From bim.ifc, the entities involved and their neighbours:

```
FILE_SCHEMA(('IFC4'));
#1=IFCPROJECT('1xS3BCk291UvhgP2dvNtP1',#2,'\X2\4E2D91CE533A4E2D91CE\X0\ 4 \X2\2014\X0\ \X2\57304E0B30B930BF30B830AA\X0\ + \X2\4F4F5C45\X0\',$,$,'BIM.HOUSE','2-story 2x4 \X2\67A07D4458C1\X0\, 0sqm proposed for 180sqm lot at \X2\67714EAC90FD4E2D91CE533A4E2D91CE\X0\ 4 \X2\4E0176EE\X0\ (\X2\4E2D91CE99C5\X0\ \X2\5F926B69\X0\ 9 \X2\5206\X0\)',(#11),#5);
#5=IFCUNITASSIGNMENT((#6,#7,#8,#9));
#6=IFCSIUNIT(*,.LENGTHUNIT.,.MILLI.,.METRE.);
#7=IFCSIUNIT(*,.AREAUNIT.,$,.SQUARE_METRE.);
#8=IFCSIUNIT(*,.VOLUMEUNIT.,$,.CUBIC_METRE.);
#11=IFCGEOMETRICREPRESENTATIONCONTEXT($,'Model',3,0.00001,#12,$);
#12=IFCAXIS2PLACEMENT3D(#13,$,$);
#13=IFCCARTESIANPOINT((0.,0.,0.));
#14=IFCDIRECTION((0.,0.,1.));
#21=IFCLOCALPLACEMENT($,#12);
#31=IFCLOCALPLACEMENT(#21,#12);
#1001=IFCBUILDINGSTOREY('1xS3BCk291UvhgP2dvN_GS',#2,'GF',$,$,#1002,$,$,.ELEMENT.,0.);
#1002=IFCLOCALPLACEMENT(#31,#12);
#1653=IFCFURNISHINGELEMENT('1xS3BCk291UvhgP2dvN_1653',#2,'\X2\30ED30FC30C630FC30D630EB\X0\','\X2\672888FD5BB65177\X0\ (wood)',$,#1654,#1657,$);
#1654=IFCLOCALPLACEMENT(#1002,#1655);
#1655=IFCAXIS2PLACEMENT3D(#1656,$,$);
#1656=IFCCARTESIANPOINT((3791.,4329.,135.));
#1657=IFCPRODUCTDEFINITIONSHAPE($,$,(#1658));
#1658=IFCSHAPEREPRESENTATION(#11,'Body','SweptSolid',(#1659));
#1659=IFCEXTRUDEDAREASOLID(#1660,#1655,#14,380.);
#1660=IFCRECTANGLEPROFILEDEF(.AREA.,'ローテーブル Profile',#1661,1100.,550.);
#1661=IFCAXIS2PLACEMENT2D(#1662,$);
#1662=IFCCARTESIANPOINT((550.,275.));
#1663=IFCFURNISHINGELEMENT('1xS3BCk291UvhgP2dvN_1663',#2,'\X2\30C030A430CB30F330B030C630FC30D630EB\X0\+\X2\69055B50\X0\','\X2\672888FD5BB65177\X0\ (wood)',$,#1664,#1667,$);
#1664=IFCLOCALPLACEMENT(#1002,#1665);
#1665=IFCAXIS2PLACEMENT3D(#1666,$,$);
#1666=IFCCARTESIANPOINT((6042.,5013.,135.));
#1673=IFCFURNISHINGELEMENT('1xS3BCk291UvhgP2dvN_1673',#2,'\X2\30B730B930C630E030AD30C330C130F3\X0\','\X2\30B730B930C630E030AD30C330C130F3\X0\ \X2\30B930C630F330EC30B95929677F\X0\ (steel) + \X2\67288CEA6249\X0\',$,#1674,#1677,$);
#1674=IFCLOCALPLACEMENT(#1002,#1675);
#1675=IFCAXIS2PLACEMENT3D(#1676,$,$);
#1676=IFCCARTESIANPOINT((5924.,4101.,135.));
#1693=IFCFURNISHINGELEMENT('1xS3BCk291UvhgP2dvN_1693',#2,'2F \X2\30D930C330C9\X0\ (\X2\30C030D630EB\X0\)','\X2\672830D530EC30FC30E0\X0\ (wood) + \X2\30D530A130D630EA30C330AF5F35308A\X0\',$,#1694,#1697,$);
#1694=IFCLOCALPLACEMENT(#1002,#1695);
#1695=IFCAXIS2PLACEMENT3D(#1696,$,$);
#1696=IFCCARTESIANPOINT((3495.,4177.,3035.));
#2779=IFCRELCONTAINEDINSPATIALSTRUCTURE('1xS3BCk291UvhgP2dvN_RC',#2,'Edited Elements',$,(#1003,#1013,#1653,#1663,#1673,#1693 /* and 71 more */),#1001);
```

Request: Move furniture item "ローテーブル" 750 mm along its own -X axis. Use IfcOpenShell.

```python
import ifcopenshell
import ifcopenshell.api.geometry
import ifcopenshell.util.placement
import ifcopenshell.util.unit

model = ifcopenshell.open("bim.ifc")
unit_scale = ifcopenshell.util.unit.calculate_unit_scale(model)

item = model.by_guid("1xS3BCk291UvhgP2dvN_1653")
matrix = ifcopenshell.util.placement.get_local_placement(item.ObjectPlacement)
matrix[:3, 3] -= matrix[:3, 0] * 0.75 / unit_scale
ifcopenshell.api.geometry.edit_object_placement(model, product=item, matrix=matrix, is_si=False)

print(ifcopenshell.util.placement.get_local_placement(item.ObjectPlacement).round(3) + 0.0)

model.write("bim_v2.ifc")
```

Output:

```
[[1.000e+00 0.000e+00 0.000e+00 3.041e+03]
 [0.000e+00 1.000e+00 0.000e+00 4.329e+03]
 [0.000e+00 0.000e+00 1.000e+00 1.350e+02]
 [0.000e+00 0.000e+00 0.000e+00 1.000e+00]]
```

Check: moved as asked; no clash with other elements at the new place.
